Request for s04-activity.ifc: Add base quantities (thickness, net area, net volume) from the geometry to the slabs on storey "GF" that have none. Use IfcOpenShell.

First a look at what the model holds.

```python
import ifcopenshell
import ifcopenshell.util.element
import ifcopenshell.util.unit

model = ifcopenshell.open("s04-activity.ifc")
print(model.schema)
for unit_type in ("LENGTHUNIT", "AREAUNIT", "VOLUMEUNIT"):
    print(unit_type, ifcopenshell.util.unit.calculate_unit_scale(model, unit_type))
storey = next(s for s in model.by_type("IfcBuildingStorey") if s.Name == "GF")
slabs = [e for e in ifcopenshell.util.element.get_decomposition(storey) if e.is_a("IfcSlab")]
for e in sorted(slabs, key=lambda e: e.id()):
    print(e.id(), e.is_a(), e.Name, list(ifcopenshell.util.element.get_psets(e, qtos_only=True)), sep=" | ")
```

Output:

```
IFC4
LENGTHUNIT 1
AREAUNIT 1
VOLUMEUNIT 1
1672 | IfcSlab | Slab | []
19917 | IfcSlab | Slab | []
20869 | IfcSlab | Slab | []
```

```python
import ifcopenshell
import ifcopenshell.api.pset
import ifcopenshell.geom
import ifcopenshell.util.element
import ifcopenshell.util.shape
import ifcopenshell.util.unit

model = ifcopenshell.open("s04-activity.ifc")
unit_scale = ifcopenshell.util.unit.calculate_unit_scale(model)
area_scale = ifcopenshell.util.unit.calculate_unit_scale(model, "AREAUNIT")
volume_scale = ifcopenshell.util.unit.calculate_unit_scale(model, "VOLUMEUNIT")
settings = ifcopenshell.geom.settings()

storey = next(s for s in model.by_type("IfcBuildingStorey") if s.Name == "GF")
slabs = [e for e in ifcopenshell.util.element.get_decomposition(storey) if e.is_a("IfcSlab")]

for e in sorted(slabs, key=lambda e: e.id()):
    if ifcopenshell.util.element.get_psets(e, qtos_only=True, should_inherit=False):
        continue
    # Geometry comes back in metres, in the element's own axes.
    shape = ifcopenshell.geom.create_shape(settings, e)
    values = {
        "Width": ifcopenshell.util.shape.get_z(shape.geometry) / unit_scale,
        "NetArea": ifcopenshell.util.shape.get_footprint_area(shape.geometry) / area_scale,
        "NetVolume": ifcopenshell.util.shape.get_volume(shape.geometry) / volume_scale,
    }
    qto = ifcopenshell.api.pset.add_qto(model, product=e, name="Qto_SlabBaseQuantities")
    ifcopenshell.api.pset.edit_qto(model, qto=qto, properties=values)
    print(e.id(), {k: round(v, 3) for k, v in values.items()})

model.write("s04-activity-out.ifc")
```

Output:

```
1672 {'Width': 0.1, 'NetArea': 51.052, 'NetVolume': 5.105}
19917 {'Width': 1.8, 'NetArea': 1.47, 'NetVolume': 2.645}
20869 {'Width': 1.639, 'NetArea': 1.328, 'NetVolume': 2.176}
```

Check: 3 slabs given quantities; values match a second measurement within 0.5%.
